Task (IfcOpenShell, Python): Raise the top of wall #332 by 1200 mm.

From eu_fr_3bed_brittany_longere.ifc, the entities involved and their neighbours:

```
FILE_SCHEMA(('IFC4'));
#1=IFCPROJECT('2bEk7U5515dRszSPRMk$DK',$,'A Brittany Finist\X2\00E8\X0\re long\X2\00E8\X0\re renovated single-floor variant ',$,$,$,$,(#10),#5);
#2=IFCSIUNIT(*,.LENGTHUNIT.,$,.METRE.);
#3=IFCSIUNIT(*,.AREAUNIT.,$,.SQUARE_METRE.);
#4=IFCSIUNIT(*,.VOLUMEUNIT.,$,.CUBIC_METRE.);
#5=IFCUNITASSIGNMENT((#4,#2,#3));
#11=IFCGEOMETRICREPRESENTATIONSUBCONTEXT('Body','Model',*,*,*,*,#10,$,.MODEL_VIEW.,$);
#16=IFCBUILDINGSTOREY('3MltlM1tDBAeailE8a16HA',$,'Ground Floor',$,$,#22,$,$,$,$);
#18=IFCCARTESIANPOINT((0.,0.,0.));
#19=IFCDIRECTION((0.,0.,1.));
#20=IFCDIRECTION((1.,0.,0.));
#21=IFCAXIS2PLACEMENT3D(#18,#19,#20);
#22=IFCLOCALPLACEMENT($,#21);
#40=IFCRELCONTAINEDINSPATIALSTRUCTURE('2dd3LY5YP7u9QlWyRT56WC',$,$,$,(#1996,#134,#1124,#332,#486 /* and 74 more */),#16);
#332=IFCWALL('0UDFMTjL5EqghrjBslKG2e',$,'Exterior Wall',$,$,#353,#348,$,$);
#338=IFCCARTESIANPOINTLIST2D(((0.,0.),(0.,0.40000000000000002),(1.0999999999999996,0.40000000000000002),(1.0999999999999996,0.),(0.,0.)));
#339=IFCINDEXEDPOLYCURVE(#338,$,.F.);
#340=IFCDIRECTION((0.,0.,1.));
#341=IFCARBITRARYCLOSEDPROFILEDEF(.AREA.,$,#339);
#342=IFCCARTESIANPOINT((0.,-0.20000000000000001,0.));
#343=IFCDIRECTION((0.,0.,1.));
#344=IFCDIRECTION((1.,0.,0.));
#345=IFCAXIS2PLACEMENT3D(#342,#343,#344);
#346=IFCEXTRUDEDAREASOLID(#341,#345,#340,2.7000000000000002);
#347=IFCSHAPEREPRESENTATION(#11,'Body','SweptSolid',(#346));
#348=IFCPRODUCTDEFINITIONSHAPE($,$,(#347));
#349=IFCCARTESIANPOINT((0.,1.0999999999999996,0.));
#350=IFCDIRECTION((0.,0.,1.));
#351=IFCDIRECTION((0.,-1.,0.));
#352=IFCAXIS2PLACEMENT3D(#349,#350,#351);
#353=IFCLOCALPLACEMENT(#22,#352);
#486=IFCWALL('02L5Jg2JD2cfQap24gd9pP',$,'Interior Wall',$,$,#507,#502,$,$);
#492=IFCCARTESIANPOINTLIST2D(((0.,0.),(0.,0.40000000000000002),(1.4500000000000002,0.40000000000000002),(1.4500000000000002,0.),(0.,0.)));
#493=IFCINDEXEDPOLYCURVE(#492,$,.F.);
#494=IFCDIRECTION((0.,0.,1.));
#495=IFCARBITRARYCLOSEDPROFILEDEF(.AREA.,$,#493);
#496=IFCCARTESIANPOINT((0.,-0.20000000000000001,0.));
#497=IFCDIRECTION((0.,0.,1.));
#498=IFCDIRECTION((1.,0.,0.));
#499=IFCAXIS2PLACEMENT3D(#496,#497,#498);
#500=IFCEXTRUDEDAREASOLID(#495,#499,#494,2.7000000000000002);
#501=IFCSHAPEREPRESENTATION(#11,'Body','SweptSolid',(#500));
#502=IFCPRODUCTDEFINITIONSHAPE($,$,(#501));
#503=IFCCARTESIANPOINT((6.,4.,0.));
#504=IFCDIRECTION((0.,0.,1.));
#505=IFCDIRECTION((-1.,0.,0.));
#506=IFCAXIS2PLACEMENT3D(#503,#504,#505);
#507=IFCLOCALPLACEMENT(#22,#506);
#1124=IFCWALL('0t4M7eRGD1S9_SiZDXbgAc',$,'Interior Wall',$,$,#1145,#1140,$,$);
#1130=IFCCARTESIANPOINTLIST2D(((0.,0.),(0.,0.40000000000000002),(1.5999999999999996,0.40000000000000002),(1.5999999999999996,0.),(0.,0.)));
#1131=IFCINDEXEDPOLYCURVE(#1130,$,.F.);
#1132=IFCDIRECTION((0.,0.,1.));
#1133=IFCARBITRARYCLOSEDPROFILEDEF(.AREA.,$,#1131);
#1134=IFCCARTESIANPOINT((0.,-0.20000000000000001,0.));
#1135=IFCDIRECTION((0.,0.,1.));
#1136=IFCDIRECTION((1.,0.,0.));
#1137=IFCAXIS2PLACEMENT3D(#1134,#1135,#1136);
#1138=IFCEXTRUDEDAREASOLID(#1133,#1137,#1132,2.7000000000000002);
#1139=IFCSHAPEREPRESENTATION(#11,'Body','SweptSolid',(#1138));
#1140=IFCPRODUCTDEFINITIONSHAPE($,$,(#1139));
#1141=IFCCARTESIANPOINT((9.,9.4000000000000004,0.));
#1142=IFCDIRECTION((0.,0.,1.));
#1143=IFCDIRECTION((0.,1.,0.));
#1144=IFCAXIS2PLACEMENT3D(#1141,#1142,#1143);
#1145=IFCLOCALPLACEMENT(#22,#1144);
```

```python
import ifcopenshell
import ifcopenshell.geom
import ifcopenshell.util.representation
import ifcopenshell.util.shape

model = ifcopenshell.open("eu_fr_3bed_brittany_longere.ifc")
settings = ifcopenshell.geom.settings()


def volume(element):
    """Net volume in cubic metres, openings subtracted."""
    shape = ifcopenshell.geom.create_shape(settings, element)
    return ifcopenshell.util.shape.get_volume(shape.geometry)


wall = model.by_guid("0UDFMTjL5EqghrjBslKG2e")
before = volume(wall)

body = ifcopenshell.util.representation.get_representation(wall, "Model", "Body")
solid = body.Items[0]
old_height = solid.Depth
solid.Depth += 1.2
after = volume(wall)

print(f"height {old_height:g} -> {solid.Depth:g}, volume {before:.3f} -> {after:.3f} m3")

model.write("eu_fr_3bed_brittany_longere_updated.ifc")
```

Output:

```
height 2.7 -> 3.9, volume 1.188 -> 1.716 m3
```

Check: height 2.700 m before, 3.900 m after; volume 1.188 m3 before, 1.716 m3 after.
